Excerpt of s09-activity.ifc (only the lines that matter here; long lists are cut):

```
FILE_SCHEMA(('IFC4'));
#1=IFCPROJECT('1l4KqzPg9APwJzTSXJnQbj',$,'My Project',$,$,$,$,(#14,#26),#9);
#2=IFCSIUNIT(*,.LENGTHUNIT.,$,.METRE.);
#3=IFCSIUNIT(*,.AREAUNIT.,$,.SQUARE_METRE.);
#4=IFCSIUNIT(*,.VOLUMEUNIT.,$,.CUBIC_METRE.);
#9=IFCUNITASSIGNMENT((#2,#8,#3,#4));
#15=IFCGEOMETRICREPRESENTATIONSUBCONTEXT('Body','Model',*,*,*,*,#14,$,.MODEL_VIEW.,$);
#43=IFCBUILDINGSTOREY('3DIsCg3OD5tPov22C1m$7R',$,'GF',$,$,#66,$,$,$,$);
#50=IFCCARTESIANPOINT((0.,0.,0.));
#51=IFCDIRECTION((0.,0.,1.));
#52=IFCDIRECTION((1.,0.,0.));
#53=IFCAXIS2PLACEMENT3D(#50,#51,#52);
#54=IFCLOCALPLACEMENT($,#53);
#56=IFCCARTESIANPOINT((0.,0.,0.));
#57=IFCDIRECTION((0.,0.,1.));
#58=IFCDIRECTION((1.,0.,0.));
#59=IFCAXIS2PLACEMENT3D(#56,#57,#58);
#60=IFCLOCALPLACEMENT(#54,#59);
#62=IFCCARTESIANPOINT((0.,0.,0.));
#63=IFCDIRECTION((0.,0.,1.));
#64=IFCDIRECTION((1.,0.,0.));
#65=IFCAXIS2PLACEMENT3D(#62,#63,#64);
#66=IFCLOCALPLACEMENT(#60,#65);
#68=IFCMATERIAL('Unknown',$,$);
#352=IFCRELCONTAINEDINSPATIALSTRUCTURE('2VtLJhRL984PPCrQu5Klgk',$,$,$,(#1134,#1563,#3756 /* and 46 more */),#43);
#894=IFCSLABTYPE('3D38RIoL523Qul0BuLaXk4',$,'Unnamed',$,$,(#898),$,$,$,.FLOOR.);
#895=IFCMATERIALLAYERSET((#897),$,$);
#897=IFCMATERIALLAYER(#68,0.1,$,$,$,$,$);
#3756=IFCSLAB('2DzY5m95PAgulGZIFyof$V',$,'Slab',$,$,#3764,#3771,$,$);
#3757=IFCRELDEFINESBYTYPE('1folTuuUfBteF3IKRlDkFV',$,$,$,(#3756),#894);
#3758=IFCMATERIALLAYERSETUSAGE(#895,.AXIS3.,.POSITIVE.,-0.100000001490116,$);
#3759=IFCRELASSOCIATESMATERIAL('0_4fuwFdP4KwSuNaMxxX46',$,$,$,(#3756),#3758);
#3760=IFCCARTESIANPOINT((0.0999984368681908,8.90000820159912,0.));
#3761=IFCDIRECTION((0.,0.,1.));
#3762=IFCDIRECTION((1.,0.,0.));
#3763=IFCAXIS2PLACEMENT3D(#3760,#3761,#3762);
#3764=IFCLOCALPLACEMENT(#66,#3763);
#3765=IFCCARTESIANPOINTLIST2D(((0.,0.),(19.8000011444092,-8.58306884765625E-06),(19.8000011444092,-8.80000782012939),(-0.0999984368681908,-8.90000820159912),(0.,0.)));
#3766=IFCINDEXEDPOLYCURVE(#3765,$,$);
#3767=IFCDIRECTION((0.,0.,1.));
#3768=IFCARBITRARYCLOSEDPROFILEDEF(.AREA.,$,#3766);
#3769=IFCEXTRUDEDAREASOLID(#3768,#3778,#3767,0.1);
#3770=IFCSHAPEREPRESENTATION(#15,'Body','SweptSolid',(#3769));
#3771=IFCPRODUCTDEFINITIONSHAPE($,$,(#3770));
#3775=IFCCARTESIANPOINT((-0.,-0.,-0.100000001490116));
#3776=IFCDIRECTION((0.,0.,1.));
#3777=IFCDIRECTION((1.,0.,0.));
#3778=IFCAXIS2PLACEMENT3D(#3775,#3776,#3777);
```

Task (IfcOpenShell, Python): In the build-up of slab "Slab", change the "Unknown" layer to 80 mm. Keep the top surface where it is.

```python
import ifcopenshell
import ifcopenshell.util.element
import ifcopenshell.util.representation

model = ifcopenshell.open("s09-activity.ifc")

layer_set = model.by_id(895)
layer = next(l for l in layer_set.MaterialLayers if l.Material and l.Material.Name == "Unknown")
change = 0.08 - layer.LayerThickness
layer.LayerThickness += change

# Geometry does not follow the layer set by itself.
slabs = [e for e in ifcopenshell.util.element.get_elements_by_material(model, layer_set) if e.is_a("IfcSlab")]
for slab in sorted(slabs, key=lambda e: e.id()):
    body = ifcopenshell.util.representation.get_representation(slab, "Model", "Body")
    solid = body.Items[0]
    old_depth = solid.Depth
    solid.Depth += change
    # Extruded upwards: lower the start of the extrusion so the top stays.
    x, y, z = solid.Position.Location.Coordinates
    solid.Position.Location = model.createIfcCartesianPoint((x, y, z - change))
    print(slab.id(), f"{old_depth:g} -> {solid.Depth:g}")

# The layers are counted up from the underside, which has moved.
for usage in {ifcopenshell.util.element.get_material(slab) for slab in slabs}:
    usage.OffsetFromReferenceLine -= change

model.write("s09-activity_updated.ifc")
```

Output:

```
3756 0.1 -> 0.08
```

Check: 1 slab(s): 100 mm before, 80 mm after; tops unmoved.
